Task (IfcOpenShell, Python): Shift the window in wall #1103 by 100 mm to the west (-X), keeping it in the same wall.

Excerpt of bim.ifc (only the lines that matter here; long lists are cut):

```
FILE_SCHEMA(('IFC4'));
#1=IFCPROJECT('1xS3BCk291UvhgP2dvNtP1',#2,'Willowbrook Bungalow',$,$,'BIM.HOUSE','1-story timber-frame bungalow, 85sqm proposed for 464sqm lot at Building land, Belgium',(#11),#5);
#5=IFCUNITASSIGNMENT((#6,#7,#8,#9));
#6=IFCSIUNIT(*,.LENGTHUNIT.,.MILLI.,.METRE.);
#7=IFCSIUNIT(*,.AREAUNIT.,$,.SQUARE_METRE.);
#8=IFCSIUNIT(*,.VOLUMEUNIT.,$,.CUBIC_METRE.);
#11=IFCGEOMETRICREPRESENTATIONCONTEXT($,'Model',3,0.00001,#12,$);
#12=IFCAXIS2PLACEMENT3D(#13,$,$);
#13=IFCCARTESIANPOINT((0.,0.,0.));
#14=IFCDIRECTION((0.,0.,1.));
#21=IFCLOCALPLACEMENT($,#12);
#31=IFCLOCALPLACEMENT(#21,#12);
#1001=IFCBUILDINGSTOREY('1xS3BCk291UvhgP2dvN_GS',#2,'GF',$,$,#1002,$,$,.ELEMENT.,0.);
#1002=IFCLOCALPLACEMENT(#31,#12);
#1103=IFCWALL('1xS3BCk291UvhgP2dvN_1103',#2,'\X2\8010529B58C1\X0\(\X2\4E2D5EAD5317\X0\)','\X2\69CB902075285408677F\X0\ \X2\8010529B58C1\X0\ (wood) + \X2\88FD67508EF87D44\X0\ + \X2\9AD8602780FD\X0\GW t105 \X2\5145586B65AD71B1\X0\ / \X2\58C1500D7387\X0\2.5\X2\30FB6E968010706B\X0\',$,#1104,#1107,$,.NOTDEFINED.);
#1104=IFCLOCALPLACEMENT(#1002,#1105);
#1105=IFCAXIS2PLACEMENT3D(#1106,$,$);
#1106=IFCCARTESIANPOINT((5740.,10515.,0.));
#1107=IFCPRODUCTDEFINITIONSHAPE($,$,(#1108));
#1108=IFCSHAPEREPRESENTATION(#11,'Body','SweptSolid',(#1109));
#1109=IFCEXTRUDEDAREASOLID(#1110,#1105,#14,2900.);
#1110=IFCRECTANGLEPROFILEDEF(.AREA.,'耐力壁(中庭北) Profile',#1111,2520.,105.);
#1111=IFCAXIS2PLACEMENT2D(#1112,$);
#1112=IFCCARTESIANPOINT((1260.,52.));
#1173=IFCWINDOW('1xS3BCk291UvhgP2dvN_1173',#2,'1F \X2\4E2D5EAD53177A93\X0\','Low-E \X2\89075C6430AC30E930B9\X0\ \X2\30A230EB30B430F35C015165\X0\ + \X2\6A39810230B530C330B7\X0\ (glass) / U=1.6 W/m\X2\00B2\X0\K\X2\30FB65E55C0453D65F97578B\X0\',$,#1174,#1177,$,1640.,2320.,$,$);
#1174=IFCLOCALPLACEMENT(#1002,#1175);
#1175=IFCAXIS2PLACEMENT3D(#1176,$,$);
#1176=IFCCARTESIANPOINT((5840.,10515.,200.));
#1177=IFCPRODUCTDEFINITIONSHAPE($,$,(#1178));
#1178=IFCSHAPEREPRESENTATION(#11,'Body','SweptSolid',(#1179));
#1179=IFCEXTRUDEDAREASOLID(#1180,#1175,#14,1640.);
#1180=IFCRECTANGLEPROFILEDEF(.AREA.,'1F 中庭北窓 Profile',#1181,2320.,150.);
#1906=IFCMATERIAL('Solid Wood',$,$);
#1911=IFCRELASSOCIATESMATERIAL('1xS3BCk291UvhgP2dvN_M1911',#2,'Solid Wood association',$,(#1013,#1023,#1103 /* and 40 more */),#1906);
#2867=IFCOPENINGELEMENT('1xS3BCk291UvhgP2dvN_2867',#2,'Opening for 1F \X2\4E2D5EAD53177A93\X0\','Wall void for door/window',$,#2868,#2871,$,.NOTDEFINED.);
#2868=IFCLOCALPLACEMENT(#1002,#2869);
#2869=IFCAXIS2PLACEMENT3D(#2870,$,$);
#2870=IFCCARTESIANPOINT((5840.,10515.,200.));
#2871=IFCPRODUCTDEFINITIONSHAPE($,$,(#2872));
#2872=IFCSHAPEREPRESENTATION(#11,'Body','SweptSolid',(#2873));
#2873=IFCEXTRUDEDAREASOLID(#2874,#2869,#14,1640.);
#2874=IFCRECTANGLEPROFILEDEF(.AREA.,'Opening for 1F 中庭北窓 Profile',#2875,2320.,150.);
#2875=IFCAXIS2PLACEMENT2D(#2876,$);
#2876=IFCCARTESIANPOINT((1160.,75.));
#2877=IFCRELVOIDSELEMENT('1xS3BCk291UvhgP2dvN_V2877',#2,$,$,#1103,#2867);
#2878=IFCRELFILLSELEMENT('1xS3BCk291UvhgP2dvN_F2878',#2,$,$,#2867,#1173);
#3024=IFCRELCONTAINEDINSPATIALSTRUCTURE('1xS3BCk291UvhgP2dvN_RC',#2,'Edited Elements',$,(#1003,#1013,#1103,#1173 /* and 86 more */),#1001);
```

```python
import ifcopenshell
import ifcopenshell.api.geometry
import ifcopenshell.util.placement

model = ifcopenshell.open("bim.ifc")

window = model.by_id(1173)
opening = window.FillsVoids[0].RelatingOpeningElement
wall = opening.VoidsElements[0].RelatingBuildingElement

wall_matrix = ifcopenshell.util.placement.get_local_placement(wall.ObjectPlacement)
shift = wall_matrix[:3, 0] * -100.0
before = ifcopenshell.util.placement.get_local_placement(window.ObjectPlacement)[:3, 3].copy()

# The window is not placed relative to its opening, so move both.
for product in (opening, window):
    matrix = ifcopenshell.util.placement.get_local_placement(product.ObjectPlacement)
    matrix[:3, 3] += shift
    ifcopenshell.api.geometry.edit_object_placement(model, product=product, matrix=matrix, is_si=False)

after = ifcopenshell.util.placement.get_local_placement(window.ObjectPlacement)[:3, 3]
print("window moved by", (after - before).round(3) + 0.0)

model.write("bim_rev.ifc")
```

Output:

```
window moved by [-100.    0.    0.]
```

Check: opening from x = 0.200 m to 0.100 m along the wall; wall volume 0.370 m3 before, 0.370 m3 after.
